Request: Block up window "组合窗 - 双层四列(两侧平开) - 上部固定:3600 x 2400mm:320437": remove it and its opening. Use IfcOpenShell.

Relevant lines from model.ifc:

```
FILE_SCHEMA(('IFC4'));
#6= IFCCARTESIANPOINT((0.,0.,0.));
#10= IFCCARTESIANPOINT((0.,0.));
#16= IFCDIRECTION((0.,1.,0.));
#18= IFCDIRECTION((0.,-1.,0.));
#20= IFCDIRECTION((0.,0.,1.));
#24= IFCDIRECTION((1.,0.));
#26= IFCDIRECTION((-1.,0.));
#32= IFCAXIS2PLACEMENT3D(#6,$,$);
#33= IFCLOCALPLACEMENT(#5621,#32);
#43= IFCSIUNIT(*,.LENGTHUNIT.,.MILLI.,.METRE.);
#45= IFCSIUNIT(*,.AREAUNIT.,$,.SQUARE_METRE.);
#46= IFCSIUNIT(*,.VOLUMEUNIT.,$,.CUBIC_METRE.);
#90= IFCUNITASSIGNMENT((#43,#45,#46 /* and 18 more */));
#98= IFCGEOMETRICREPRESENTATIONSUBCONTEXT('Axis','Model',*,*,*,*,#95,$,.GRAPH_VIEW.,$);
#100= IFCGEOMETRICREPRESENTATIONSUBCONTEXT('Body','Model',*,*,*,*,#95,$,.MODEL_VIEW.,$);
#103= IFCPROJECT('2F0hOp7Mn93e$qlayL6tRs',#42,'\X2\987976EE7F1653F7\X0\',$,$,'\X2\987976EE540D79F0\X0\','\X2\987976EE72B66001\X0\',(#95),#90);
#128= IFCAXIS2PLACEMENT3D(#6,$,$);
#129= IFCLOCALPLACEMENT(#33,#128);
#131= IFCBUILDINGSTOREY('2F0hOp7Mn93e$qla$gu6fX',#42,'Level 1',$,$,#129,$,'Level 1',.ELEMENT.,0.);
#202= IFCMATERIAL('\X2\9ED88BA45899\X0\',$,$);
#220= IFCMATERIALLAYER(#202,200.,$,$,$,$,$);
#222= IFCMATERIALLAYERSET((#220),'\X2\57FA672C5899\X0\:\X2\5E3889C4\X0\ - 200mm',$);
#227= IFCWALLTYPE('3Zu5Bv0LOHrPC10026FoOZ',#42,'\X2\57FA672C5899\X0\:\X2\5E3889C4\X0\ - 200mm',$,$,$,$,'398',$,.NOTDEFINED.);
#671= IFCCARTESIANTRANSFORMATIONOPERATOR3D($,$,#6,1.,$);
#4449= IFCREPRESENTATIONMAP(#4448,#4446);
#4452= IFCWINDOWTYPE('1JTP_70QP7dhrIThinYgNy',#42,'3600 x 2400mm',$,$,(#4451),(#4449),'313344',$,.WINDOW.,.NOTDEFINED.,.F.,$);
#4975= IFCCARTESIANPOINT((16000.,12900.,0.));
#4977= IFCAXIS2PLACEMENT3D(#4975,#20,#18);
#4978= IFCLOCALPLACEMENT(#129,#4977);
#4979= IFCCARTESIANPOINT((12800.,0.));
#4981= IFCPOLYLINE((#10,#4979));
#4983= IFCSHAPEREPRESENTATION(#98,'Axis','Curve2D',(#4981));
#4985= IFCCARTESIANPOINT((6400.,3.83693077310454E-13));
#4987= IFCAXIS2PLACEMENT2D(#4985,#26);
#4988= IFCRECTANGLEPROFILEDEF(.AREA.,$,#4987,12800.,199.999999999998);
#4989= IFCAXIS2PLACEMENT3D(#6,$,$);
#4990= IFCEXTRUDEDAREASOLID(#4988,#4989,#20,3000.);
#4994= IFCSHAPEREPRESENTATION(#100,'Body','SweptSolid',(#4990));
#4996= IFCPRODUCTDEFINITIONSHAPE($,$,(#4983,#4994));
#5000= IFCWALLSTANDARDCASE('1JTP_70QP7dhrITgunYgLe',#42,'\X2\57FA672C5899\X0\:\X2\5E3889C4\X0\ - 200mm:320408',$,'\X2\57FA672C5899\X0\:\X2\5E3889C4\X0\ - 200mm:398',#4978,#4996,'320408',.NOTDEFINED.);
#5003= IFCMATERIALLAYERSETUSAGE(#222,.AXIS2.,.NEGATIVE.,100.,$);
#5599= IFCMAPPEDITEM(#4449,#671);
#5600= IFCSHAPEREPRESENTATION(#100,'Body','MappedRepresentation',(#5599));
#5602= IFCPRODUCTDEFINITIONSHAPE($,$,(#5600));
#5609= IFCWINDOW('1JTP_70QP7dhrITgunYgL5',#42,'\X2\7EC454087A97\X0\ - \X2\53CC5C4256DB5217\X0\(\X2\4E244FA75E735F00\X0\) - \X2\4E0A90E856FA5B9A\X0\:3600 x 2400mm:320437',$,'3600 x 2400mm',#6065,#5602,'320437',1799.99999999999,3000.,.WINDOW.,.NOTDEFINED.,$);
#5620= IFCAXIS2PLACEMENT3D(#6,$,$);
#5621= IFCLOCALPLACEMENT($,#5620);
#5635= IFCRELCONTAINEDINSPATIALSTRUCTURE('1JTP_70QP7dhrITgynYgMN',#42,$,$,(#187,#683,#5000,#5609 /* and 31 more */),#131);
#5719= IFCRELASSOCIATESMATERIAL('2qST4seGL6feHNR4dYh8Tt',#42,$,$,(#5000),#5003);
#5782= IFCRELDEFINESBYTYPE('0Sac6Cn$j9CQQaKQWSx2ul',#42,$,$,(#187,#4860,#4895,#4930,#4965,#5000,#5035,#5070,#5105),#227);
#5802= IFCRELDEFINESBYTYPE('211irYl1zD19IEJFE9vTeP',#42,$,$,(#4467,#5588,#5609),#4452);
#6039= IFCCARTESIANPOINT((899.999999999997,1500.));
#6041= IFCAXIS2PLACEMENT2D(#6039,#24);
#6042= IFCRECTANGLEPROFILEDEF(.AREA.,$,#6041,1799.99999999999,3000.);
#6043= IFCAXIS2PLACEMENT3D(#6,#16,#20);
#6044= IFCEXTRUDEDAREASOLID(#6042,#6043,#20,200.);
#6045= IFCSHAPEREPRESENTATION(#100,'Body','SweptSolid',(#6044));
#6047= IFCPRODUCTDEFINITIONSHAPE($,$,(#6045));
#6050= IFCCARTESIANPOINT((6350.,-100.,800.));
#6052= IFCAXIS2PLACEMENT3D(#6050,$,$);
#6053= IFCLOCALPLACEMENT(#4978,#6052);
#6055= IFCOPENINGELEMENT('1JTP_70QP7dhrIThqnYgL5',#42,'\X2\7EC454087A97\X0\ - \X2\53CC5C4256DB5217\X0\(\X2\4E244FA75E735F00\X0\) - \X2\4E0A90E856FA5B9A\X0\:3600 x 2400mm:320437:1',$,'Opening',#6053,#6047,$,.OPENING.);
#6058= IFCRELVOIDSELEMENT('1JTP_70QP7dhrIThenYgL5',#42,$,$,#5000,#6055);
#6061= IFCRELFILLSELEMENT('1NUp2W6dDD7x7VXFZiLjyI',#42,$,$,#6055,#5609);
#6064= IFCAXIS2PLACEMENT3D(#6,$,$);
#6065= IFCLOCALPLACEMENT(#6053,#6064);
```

```python
import ifcopenshell
import ifcopenshell.api.feature
import ifcopenshell.api.root
import ifcopenshell.geom
import ifcopenshell.util.shape

model = ifcopenshell.open("model.ifc")
settings = ifcopenshell.geom.settings()


def volume(element):
    """Net volume in cubic metres, openings subtracted."""
    shape = ifcopenshell.geom.create_shape(settings, element)
    return ifcopenshell.util.shape.get_volume(shape.geometry)


window = model.by_guid("1JTP_70QP7dhrITgunYgL5")
opening = window.FillsVoids[0].RelatingOpeningElement
wall = opening.VoidsElements[0].RelatingBuildingElement
before = volume(wall)

ifcopenshell.api.root.remove_product(model, product=window)
ifcopenshell.api.feature.remove_feature(model, feature=opening)

after = volume(wall)

print(f"wall volume {before:.3f} -> {after:.3f} m3")

model.write("model-out.ifc")
```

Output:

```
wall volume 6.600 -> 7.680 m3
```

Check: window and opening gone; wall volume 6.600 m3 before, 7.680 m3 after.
